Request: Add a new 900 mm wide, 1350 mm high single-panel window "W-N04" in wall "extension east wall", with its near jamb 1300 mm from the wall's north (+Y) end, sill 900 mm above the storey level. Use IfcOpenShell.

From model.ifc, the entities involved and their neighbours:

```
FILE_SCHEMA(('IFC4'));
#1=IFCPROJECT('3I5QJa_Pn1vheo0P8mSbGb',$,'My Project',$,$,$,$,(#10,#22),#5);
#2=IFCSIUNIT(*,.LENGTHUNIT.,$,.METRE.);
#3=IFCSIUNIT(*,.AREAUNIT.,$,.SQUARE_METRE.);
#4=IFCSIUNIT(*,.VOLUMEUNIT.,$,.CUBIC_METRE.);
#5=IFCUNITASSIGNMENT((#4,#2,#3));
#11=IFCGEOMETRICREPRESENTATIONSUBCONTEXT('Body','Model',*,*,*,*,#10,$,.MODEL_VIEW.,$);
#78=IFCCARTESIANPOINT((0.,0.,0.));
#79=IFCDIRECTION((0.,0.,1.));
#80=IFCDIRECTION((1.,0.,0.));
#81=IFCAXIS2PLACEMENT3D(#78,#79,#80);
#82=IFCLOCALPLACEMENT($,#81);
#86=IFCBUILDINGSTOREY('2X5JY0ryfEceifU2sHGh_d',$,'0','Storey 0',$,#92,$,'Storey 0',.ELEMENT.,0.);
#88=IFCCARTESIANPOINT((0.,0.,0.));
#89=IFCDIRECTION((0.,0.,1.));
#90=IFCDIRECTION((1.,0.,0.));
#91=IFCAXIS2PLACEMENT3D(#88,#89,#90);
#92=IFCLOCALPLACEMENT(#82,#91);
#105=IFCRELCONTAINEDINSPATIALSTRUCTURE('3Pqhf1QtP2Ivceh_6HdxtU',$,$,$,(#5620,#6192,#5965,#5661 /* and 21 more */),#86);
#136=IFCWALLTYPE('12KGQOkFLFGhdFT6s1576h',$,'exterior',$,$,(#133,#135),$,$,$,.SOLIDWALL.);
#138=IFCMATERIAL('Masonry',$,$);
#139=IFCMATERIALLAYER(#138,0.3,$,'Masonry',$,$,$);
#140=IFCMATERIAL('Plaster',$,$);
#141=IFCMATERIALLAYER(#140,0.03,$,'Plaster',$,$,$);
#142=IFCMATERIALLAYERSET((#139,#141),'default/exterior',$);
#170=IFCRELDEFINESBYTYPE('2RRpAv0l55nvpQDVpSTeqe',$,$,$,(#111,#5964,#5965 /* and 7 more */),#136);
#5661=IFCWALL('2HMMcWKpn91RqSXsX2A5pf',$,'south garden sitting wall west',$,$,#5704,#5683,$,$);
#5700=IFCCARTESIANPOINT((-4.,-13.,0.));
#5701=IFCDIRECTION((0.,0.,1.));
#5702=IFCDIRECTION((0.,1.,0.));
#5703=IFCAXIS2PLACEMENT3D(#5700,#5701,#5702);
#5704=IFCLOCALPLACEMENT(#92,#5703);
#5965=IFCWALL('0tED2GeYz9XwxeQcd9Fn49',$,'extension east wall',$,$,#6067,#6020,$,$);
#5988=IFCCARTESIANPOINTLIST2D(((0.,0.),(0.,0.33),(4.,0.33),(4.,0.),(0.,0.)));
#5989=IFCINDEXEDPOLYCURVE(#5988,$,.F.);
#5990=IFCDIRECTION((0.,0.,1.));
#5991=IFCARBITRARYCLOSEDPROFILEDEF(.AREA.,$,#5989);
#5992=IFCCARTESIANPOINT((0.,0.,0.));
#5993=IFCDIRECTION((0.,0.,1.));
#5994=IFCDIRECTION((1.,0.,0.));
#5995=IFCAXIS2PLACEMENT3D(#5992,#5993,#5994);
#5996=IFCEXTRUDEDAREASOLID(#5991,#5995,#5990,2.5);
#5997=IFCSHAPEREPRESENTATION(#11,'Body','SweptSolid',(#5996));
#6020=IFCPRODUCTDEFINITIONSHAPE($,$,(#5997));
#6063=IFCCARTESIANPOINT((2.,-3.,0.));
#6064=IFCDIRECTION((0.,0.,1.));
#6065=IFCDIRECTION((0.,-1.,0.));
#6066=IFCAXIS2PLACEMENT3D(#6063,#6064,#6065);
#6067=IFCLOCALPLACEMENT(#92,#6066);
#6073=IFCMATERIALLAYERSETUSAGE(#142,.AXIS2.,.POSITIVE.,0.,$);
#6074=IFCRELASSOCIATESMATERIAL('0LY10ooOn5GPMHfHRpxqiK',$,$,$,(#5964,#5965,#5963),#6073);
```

```python
import numpy as np
import ifcopenshell
import ifcopenshell.api.feature
import ifcopenshell.api.geometry
import ifcopenshell.api.root
import ifcopenshell.api.spatial
import ifcopenshell.geom
import ifcopenshell.util.element
import ifcopenshell.util.placement
import ifcopenshell.util.representation
import ifcopenshell.util.shape
import ifcopenshell.util.unit

model = ifcopenshell.open("model.ifc")
unit_scale = ifcopenshell.util.unit.calculate_unit_scale(model)
settings = ifcopenshell.geom.settings()


def volume(element):
    """Net volume in cubic metres, openings subtracted."""
    shape = ifcopenshell.geom.create_shape(settings, element)
    return ifcopenshell.util.shape.get_volume(shape.geometry)


wall = model.by_guid("0tED2GeYz9XwxeQcd9Fn49")
storey = ifcopenshell.util.element.get_container(wall, ifc_class="IfcBuildingStorey")
context = ifcopenshell.util.representation.get_context(model, "Model", "Body", "MODEL_VIEW")
before = volume(wall)

width, height, from_end, sill = 0.9, 1.35, 1.3, 0.9  # metres

# The wall runs along its own X axis, and the end named is its -X end.
wall_shape = ifcopenshell.geom.create_shape(settings, wall)
x, y, z = ifcopenshell.util.shape.get_vertices(wall_shape.geometry).T
start = x.min() + from_end
face, thickness = float(y.min()), float(y.max() - y.min())
wall_matrix = ifcopenshell.util.placement.get_local_placement(wall.ObjectPlacement)
level = ifcopenshell.util.placement.get_local_placement(storey.ObjectPlacement)[2, 3]


def in_wall(x, y):
    """Placement at x, y metres in the wall's axes, at sill height."""
    matrix = wall_matrix.copy()
    matrix[:, 3] = wall_matrix @ np.array([x / unit_scale, y / unit_scale, 0.0, 1.0])
    matrix[2, 3] = level + sill / unit_scale
    return matrix


# Opening: a box that overshoots both wall faces by 50 mm.
opening = ifcopenshell.api.root.create_entity(model, ifc_class="IfcOpeningElement", predefined_type="OPENING")
box = ifcopenshell.api.geometry.add_wall_representation(
    model, context=context, length=width, height=height, thickness=thickness + 0.1
)
ifcopenshell.api.geometry.assign_representation(model, product=opening, representation=box)
ifcopenshell.api.geometry.edit_object_placement(model, product=opening, matrix=in_wall(start, face - 0.05), is_si=False)
ifcopenshell.api.feature.add_feature(model, feature=opening, element=wall)

window = ifcopenshell.api.root.create_entity(model, ifc_class="IfcWindow", name="W-N04", predefined_type="WINDOW")
window.OverallWidth, window.OverallHeight = width / unit_scale, height / unit_scale
window.PartitioningType = "SINGLE_PANEL"
body = ifcopenshell.api.geometry.add_window_representation(
    model,
    context=context,
    overall_width=window.OverallWidth,
    overall_height=window.OverallHeight,
    partition_type="SINGLE_PANEL",
)
ifcopenshell.api.geometry.assign_representation(model, product=window, representation=body)
ifcopenshell.api.spatial.assign_container(model, products=[window], relating_structure=storey)
ifcopenshell.api.feature.add_filling(model, opening=opening, element=window)

# Centre the window in the wall's thickness.
ifcopenshell.api.geometry.edit_object_placement(model, product=window, matrix=in_wall(start, face), is_si=False)
window_shape = ifcopenshell.geom.create_shape(settings, window)
depth = ifcopenshell.util.shape.get_vertices(window_shape.geometry)[:, 1]
offset = face + thickness / 2 - (depth.min() + depth.max()) / 2
ifcopenshell.api.geometry.edit_object_placement(model, product=window, matrix=in_wall(start, offset), is_si=False)

after = volume(wall)

print(f"wall volume {before:.3f} -> {after:.3f} m3")

model.write("model_edited.ifc")
```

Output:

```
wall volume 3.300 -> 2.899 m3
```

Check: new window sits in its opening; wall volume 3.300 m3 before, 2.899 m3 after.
